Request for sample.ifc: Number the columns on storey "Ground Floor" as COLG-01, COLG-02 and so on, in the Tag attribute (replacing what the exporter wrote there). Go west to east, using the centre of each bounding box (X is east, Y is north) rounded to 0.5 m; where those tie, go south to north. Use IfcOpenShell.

First a look at what the model holds.

```python
import ifcopenshell
import ifcopenshell.util.element
import ifcopenshell.util.placement

model = ifcopenshell.open("sample.ifc")
print(model.schema)
storey = next(s for s in model.by_type("IfcBuildingStorey") if s.Name == "Ground Floor")
columns = [e for e in ifcopenshell.util.element.get_decomposition(storey) if e.is_a("IfcColumn")]
for e in sorted(columns, key=lambda e: e.id()):
    origin = ifcopenshell.util.placement.get_local_placement(e.ObjectPlacement)[:3, 3]
    print(e.id(), e.Tag, e.Name, origin.round(2) + 0.0, sep=" | ")
```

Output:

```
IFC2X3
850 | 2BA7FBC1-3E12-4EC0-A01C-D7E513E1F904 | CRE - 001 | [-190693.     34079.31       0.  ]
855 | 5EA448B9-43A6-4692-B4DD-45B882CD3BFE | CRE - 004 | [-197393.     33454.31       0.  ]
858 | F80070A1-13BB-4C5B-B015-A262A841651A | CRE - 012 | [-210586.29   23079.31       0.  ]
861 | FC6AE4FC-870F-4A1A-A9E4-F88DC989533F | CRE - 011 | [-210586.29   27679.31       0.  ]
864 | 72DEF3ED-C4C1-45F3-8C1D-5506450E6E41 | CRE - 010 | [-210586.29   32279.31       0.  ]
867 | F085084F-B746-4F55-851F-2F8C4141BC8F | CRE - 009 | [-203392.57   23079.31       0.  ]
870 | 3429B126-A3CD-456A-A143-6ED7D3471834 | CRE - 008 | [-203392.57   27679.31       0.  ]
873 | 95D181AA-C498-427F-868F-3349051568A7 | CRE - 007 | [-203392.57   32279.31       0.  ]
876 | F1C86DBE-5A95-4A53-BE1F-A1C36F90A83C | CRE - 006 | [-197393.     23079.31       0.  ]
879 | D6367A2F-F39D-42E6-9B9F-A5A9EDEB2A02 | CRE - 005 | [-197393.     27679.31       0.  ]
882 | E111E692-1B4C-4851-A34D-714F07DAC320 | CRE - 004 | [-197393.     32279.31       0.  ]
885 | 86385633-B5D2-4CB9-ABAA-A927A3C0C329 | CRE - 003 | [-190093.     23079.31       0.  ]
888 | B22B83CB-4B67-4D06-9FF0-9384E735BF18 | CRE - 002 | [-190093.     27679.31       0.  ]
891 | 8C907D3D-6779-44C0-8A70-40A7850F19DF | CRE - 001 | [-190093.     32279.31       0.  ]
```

```python
import ifcopenshell
import ifcopenshell.geom
import ifcopenshell.util.element
import ifcopenshell.util.shape

model = ifcopenshell.open("sample.ifc")
settings = ifcopenshell.geom.settings()
settings.set("use-world-coords", True)


def centre(element):
    shape = ifcopenshell.geom.create_shape(settings, element)
    return ifcopenshell.util.shape.get_bbox_centroid(shape.geometry)


storey = next(s for s in model.by_type("IfcBuildingStorey") if s.Name == "Ground Floor")
columns = [e for e in ifcopenshell.util.element.get_decomposition(storey) if e.is_a("IfcColumn")]

# Insertion points can sit at a corner or the storey origin, so sort by the geometry (in metres).
centres = {e: centre(e) for e in columns}
columns.sort(key=lambda e: (round(centres[e][0] / 0.5), centres[e][1]))

for i, e in enumerate(columns, start=1):
    number = f"COLG-{i:02d}"
    e.Tag = number
    print(e.id(), number)

model.write("sample-out.ifc")
```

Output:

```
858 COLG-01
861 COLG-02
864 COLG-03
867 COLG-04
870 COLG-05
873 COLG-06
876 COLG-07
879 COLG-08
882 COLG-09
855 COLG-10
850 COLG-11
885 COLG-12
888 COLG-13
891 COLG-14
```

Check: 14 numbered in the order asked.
